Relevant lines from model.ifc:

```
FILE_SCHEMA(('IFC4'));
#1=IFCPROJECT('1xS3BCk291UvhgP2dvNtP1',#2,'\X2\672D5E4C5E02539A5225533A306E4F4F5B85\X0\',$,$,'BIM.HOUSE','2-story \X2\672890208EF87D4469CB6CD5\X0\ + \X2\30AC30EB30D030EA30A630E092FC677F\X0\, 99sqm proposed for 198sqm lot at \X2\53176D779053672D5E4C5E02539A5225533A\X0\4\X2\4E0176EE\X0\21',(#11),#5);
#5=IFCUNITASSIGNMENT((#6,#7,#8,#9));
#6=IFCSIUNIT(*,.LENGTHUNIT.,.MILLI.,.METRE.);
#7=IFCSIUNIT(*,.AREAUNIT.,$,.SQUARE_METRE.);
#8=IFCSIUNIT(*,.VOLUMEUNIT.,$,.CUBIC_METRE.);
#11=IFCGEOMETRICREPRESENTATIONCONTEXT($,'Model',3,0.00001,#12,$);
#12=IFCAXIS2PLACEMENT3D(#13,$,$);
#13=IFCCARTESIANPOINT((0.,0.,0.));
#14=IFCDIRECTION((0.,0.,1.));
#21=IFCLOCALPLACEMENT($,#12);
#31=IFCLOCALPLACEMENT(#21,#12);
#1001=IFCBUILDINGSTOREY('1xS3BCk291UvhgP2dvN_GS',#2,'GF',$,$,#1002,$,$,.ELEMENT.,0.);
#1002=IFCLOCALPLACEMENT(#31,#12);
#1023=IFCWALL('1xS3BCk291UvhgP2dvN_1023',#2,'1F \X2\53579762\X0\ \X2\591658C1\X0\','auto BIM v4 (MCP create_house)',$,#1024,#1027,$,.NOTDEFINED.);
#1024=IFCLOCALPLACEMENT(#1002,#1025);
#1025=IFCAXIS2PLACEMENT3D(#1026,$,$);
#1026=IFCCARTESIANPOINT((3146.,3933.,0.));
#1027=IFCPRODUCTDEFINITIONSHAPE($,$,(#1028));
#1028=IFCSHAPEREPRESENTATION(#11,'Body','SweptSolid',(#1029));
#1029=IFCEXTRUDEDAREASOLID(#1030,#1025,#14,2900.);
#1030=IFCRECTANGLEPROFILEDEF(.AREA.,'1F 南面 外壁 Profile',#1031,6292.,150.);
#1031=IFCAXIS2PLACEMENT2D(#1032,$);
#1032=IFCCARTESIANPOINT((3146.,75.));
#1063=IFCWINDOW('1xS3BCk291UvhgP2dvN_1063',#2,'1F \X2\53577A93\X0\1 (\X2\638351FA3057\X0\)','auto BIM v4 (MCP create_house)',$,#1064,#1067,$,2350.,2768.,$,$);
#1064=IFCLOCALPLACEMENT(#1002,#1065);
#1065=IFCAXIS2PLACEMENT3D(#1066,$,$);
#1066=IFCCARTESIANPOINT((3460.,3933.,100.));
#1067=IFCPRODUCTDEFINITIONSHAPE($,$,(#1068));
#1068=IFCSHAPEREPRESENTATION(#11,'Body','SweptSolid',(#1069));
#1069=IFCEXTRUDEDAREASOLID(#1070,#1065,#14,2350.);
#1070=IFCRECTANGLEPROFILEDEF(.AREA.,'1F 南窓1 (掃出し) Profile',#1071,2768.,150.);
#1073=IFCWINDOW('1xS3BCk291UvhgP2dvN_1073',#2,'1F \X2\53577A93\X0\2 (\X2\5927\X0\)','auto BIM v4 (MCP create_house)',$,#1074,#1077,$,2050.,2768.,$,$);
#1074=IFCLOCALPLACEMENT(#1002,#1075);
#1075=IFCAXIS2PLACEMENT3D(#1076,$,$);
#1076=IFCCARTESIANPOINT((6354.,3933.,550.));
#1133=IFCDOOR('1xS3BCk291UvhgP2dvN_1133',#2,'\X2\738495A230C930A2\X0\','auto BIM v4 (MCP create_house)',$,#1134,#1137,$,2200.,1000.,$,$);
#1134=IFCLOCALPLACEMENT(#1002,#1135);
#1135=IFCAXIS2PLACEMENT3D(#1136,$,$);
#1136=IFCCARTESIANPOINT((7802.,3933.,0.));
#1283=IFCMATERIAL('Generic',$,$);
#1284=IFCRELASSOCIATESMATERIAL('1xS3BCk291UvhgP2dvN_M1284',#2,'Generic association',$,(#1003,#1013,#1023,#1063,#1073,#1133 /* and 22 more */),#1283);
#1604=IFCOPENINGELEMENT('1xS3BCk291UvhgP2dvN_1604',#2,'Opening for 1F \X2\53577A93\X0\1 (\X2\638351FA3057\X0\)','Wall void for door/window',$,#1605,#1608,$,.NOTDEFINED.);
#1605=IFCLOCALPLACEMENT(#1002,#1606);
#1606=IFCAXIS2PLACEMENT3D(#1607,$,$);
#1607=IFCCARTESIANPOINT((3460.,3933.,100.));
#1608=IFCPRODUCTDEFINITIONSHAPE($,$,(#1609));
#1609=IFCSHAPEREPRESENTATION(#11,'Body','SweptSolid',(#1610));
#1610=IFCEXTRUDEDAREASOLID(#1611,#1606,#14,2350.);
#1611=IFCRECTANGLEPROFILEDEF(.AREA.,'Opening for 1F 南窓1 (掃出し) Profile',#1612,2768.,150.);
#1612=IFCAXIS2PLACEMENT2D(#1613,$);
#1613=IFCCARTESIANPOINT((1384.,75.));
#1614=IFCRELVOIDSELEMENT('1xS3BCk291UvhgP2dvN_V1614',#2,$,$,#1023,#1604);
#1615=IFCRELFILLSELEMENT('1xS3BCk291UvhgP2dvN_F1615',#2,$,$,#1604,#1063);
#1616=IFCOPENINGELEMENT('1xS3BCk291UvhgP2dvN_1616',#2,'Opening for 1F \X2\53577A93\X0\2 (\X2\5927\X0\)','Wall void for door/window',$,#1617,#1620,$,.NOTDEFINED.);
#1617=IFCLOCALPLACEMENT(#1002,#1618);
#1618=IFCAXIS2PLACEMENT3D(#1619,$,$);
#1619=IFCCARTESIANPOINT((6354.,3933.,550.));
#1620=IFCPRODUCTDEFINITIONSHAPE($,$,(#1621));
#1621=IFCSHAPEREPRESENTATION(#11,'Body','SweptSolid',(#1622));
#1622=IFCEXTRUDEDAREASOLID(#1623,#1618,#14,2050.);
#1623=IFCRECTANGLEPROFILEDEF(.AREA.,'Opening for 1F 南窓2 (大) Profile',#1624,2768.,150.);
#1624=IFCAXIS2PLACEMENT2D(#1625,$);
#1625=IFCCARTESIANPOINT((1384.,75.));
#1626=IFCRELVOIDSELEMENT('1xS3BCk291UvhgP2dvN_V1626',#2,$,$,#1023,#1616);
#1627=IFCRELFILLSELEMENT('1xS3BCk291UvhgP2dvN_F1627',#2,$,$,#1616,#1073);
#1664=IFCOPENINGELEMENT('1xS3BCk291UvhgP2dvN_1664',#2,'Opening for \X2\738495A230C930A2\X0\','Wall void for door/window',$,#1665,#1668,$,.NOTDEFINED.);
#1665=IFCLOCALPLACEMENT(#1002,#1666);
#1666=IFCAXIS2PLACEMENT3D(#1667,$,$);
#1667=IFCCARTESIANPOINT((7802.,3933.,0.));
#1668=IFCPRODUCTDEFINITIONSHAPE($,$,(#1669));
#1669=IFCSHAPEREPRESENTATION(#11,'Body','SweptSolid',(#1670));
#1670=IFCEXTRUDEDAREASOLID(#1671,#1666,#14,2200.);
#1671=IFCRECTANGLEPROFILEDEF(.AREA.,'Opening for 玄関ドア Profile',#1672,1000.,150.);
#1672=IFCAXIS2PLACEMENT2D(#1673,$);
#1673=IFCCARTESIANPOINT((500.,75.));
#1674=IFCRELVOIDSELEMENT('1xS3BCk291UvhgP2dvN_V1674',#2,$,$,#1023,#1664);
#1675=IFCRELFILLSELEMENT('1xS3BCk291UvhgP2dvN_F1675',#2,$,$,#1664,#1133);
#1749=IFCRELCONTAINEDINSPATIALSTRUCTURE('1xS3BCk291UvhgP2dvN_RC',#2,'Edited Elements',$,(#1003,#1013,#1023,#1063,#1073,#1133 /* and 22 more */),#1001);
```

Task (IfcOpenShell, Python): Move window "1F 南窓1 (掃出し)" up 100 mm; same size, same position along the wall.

```python
import numpy as np
import ifcopenshell
import ifcopenshell.api.geometry
import ifcopenshell.util.placement
import ifcopenshell.util.unit

model = ifcopenshell.open("model.ifc")
unit_scale = ifcopenshell.util.unit.calculate_unit_scale(model)

window = model.by_guid("1xS3BCk291UvhgP2dvN_1063")
opening = window.FillsVoids[0].RelatingOpeningElement
dz = 0.1 / unit_scale

shift = np.array([0.0, 0.0, dz])
# The window is not placed relative to its opening, so move both.
for product in (opening, window):
    matrix = ifcopenshell.util.placement.get_local_placement(product.ObjectPlacement)
    matrix[:3, 3] += shift
    ifcopenshell.api.geometry.edit_object_placement(model, product=product, matrix=matrix, is_si=False)

print(f"moved by {dz * unit_scale:+.3f} m")

model.write("model_v2.ifc")
```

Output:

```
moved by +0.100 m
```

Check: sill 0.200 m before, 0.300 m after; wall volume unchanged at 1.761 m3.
